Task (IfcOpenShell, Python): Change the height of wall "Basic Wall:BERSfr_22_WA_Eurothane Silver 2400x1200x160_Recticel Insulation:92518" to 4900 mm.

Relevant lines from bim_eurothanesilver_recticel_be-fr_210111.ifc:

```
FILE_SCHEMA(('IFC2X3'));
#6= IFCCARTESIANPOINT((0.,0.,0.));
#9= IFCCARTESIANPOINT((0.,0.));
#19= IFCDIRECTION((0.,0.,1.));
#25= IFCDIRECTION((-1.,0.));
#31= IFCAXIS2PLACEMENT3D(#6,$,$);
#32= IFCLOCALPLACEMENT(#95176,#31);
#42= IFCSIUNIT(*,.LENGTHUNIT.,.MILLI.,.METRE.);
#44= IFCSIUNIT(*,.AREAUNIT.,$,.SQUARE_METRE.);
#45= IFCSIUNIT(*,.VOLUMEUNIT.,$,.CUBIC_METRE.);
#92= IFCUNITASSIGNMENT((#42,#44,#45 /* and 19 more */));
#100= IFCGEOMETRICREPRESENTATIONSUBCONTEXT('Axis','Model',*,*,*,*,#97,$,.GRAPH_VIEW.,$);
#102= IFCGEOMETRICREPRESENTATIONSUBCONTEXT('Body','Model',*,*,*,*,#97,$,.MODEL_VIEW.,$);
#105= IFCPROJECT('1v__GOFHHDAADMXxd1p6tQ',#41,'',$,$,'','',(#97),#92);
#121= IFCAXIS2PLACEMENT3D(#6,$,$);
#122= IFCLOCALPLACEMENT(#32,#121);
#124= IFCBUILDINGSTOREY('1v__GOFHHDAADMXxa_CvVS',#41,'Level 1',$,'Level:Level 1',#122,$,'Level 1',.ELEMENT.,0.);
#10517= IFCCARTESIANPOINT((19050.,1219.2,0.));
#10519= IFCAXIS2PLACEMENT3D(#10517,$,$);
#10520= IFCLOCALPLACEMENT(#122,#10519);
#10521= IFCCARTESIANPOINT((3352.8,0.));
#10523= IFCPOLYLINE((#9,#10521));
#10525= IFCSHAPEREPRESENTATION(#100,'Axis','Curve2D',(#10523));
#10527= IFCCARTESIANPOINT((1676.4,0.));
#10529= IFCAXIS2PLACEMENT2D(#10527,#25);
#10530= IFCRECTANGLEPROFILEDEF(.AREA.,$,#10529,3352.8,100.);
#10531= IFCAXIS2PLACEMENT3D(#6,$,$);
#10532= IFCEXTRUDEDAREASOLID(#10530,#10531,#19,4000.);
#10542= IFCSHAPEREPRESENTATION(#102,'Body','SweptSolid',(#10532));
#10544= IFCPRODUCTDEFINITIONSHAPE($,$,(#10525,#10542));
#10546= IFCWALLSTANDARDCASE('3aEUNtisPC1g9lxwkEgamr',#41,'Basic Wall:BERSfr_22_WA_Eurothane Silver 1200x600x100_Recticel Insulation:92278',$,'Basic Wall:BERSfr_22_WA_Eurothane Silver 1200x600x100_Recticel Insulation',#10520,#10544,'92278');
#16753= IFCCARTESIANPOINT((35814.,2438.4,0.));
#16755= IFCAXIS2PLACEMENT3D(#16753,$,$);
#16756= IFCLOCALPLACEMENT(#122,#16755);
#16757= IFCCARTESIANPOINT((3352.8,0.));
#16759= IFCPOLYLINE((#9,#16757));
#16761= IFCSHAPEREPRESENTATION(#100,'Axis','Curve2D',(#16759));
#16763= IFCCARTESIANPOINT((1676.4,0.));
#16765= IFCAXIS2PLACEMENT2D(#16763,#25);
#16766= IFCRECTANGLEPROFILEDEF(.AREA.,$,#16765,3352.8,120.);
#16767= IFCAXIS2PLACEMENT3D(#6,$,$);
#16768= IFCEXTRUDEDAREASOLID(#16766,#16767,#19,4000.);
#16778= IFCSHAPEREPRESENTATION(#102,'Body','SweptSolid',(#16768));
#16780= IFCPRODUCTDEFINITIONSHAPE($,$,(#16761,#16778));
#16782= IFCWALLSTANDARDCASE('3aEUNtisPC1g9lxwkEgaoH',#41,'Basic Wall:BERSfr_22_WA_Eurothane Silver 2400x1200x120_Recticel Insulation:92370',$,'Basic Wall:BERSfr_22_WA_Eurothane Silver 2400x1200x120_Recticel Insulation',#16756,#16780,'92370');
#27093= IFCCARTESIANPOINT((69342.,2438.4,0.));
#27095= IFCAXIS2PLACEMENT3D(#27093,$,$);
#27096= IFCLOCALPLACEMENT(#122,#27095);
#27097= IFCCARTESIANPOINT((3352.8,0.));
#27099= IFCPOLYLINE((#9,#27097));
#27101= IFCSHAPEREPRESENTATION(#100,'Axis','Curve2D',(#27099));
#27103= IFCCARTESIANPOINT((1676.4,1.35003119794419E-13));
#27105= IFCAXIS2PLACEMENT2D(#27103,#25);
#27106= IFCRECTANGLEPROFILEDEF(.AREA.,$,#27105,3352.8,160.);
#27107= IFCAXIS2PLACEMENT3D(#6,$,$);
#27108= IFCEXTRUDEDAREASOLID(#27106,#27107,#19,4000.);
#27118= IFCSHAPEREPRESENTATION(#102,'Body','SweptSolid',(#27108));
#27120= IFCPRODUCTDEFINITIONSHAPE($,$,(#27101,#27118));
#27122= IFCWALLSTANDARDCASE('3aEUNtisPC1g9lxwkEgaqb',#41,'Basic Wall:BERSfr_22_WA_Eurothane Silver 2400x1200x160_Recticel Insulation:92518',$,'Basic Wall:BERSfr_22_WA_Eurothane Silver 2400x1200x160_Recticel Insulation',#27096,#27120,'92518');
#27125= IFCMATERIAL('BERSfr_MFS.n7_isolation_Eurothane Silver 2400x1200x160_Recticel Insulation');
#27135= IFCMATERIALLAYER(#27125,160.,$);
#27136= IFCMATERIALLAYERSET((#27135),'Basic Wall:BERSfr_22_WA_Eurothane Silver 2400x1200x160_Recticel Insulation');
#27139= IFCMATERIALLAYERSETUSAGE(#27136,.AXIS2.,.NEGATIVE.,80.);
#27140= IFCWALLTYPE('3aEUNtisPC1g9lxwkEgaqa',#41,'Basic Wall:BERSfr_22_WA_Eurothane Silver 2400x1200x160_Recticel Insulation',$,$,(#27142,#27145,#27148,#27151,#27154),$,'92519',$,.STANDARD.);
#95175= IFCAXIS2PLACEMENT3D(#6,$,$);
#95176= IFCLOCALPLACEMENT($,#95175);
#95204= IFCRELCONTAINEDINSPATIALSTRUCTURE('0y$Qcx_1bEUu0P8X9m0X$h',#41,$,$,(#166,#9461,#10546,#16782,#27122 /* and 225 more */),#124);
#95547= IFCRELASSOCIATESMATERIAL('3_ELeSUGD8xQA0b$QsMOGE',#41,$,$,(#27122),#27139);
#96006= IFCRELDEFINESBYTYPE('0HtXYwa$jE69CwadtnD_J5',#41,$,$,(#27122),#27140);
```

```python
import ifcopenshell
import ifcopenshell.geom
import ifcopenshell.util.representation
import ifcopenshell.util.shape

model = ifcopenshell.open("bim_eurothanesilver_recticel_be-fr_210111.ifc")
settings = ifcopenshell.geom.settings()


def volume(element):
    """Net volume in cubic metres, openings subtracted."""
    shape = ifcopenshell.geom.create_shape(settings, element)
    return ifcopenshell.util.shape.get_volume(shape.geometry)


wall = model.by_guid("3aEUNtisPC1g9lxwkEgaqb")
before = volume(wall)

body = ifcopenshell.util.representation.get_representation(wall, "Model", "Body")
solid = body.Items[0]
old_height = solid.Depth
solid.Depth = 4900.0
after = volume(wall)

print(f"height {old_height:g} -> {solid.Depth:g}, volume {before:.3f} -> {after:.3f} m3")

model.write("bim_eurothanesilver_recticel_be-fr_210111_rev.ifc")
```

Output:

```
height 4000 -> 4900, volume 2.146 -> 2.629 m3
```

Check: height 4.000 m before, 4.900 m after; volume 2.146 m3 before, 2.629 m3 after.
